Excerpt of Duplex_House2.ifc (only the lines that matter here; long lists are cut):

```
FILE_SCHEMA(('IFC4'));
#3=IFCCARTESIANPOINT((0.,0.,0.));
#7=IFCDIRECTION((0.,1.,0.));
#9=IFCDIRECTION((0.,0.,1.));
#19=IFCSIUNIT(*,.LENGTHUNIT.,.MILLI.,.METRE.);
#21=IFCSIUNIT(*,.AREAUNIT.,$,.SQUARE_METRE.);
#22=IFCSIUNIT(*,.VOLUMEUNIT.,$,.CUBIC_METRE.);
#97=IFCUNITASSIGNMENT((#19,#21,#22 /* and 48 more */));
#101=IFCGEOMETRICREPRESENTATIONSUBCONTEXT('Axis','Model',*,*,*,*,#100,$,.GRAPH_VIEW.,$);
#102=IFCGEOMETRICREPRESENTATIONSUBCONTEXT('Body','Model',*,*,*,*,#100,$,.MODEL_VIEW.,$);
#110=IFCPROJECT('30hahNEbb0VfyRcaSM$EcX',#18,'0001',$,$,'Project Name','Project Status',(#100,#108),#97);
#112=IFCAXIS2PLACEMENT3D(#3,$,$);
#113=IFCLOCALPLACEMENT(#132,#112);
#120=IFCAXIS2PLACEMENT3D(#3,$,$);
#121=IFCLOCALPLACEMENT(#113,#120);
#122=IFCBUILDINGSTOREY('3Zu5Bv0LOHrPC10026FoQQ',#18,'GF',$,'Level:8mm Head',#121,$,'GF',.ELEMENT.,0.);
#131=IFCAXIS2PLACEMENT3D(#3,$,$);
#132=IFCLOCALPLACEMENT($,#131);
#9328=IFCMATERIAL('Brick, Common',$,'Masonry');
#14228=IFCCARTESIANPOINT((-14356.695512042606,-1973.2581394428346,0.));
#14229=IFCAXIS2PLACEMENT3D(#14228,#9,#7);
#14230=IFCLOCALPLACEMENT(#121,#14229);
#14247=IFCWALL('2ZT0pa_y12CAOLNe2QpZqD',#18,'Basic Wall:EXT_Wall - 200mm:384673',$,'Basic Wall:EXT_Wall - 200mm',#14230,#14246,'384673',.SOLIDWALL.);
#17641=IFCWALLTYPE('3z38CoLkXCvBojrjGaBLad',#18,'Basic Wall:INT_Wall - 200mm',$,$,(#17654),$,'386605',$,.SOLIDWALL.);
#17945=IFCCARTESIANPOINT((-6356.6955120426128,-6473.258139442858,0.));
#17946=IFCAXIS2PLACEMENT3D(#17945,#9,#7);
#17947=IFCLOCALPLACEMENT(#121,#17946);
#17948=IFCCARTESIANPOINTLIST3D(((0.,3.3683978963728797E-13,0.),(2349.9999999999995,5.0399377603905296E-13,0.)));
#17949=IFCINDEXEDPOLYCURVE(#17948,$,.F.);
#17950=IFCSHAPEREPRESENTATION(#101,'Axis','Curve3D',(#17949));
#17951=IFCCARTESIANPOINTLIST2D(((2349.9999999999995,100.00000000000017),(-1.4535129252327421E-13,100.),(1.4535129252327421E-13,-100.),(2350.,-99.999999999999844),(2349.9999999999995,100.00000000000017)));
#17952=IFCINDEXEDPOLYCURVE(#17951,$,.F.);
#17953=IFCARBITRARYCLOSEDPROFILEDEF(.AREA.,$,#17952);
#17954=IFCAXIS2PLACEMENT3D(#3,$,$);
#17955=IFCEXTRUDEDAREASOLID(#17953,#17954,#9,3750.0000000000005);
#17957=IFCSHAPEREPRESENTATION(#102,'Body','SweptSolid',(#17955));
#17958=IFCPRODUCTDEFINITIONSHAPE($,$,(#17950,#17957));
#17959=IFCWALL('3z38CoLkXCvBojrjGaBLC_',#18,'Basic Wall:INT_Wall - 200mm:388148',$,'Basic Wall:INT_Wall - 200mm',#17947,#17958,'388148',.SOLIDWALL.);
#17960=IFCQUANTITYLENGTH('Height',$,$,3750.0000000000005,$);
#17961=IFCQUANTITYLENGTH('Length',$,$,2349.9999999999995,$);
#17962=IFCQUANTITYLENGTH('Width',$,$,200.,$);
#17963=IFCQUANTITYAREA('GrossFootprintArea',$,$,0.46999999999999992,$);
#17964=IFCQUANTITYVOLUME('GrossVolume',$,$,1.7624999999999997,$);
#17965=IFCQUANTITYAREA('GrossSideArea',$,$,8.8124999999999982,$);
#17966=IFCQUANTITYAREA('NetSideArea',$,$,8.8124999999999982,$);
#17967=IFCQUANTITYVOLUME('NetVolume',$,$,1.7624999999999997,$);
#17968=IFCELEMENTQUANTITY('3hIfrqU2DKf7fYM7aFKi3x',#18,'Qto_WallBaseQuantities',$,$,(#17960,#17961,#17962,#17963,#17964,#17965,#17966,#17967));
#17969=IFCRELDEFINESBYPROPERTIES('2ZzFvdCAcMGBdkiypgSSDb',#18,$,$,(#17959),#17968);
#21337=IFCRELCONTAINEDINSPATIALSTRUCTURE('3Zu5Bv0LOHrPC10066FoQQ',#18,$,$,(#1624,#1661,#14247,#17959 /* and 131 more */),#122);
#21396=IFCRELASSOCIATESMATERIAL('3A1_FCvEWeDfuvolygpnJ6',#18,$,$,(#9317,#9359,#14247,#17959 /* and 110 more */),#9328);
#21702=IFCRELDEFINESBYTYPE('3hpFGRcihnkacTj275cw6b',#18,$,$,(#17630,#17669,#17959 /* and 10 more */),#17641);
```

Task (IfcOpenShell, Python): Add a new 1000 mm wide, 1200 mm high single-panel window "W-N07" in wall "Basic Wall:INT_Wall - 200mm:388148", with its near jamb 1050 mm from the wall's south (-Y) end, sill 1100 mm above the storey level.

```python
import numpy as np
import ifcopenshell
import ifcopenshell.api.feature
import ifcopenshell.api.geometry
import ifcopenshell.api.pset
import ifcopenshell.api.root
import ifcopenshell.api.spatial
import ifcopenshell.geom
import ifcopenshell.util.element
import ifcopenshell.util.placement
import ifcopenshell.util.representation
import ifcopenshell.util.shape
import ifcopenshell.util.unit

model = ifcopenshell.open("Duplex_House2.ifc")
unit_scale = ifcopenshell.util.unit.calculate_unit_scale(model)
area_scale = ifcopenshell.util.unit.calculate_unit_scale(model, "AREAUNIT")
volume_scale = ifcopenshell.util.unit.calculate_unit_scale(model, "VOLUMEUNIT")
settings = ifcopenshell.geom.settings()


def volume(element):
    """Net volume in cubic metres, openings subtracted."""
    shape = ifcopenshell.geom.create_shape(settings, element)
    return ifcopenshell.util.shape.get_volume(shape.geometry)


wall = model.by_guid("3z38CoLkXCvBojrjGaBLC_")
storey = ifcopenshell.util.element.get_container(wall, ifc_class="IfcBuildingStorey")
context = ifcopenshell.util.representation.get_context(model, "Model", "Body", "MODEL_VIEW")
before = volume(wall)

width, height, from_end, sill = 1, 1.2, 1.05, 1.1  # metres

# The wall runs along its own X axis, and the end named is its -X end.
wall_shape = ifcopenshell.geom.create_shape(settings, wall)
x, y, z = ifcopenshell.util.shape.get_vertices(wall_shape.geometry).T
start = x.min() + from_end
face, thickness = float(y.min()), float(y.max() - y.min())
wall_matrix = ifcopenshell.util.placement.get_local_placement(wall.ObjectPlacement)
level = ifcopenshell.util.placement.get_local_placement(storey.ObjectPlacement)[2, 3]


def in_wall(x, y):
    """Placement at x, y metres in the wall's axes, at sill height."""
    matrix = wall_matrix.copy()
    matrix[:, 3] = wall_matrix @ np.array([x / unit_scale, y / unit_scale, 0.0, 1.0])
    matrix[2, 3] = level + sill / unit_scale
    return matrix


# Opening: a box that overshoots both wall faces by 50 mm.
opening = ifcopenshell.api.root.create_entity(model, ifc_class="IfcOpeningElement", predefined_type="OPENING")
box = ifcopenshell.api.geometry.add_wall_representation(
    model, context=context, length=width, height=height, thickness=thickness + 0.1
)
ifcopenshell.api.geometry.assign_representation(model, product=opening, representation=box)
ifcopenshell.api.geometry.edit_object_placement(model, product=opening, matrix=in_wall(start, face - 0.05), is_si=False)
ifcopenshell.api.feature.add_feature(model, feature=opening, element=wall)

window = ifcopenshell.api.root.create_entity(model, ifc_class="IfcWindow", name="W-N07", predefined_type="WINDOW")
window.OverallWidth, window.OverallHeight = width / unit_scale, height / unit_scale
window.PartitioningType = "SINGLE_PANEL"
body = ifcopenshell.api.geometry.add_window_representation(
    model,
    context=context,
    overall_width=window.OverallWidth,
    overall_height=window.OverallHeight,
    partition_type="SINGLE_PANEL",
)
ifcopenshell.api.geometry.assign_representation(model, product=window, representation=body)
ifcopenshell.api.spatial.assign_container(model, products=[window], relating_structure=storey)
ifcopenshell.api.feature.add_filling(model, opening=opening, element=window)

# Centre the window in the wall's thickness.
ifcopenshell.api.geometry.edit_object_placement(model, product=window, matrix=in_wall(start, face), is_si=False)
window_shape = ifcopenshell.geom.create_shape(settings, window)
depth = ifcopenshell.util.shape.get_vertices(window_shape.geometry)[:, 1]
offset = face + thickness / 2 - (depth.min() + depth.max()) / 2
ifcopenshell.api.geometry.edit_object_placement(model, product=window, matrix=in_wall(start, offset), is_si=False)

after = volume(wall)

# Update the wall's stored quantities.
qto = model.by_id(ifcopenshell.util.element.get_pset(wall, "Qto_WallBaseQuantities", should_inherit=False)["id"])
ifcopenshell.api.pset.edit_qto(model, qto=qto, properties={
    "NetSideArea": after / thickness / area_scale,
    "NetVolume": after / volume_scale,
})

print(f"wall volume {before:.3f} -> {after:.3f} m3")

model.write("Duplex_House2_edited.ifc")
```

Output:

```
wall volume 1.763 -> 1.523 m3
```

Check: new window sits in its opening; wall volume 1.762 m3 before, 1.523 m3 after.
